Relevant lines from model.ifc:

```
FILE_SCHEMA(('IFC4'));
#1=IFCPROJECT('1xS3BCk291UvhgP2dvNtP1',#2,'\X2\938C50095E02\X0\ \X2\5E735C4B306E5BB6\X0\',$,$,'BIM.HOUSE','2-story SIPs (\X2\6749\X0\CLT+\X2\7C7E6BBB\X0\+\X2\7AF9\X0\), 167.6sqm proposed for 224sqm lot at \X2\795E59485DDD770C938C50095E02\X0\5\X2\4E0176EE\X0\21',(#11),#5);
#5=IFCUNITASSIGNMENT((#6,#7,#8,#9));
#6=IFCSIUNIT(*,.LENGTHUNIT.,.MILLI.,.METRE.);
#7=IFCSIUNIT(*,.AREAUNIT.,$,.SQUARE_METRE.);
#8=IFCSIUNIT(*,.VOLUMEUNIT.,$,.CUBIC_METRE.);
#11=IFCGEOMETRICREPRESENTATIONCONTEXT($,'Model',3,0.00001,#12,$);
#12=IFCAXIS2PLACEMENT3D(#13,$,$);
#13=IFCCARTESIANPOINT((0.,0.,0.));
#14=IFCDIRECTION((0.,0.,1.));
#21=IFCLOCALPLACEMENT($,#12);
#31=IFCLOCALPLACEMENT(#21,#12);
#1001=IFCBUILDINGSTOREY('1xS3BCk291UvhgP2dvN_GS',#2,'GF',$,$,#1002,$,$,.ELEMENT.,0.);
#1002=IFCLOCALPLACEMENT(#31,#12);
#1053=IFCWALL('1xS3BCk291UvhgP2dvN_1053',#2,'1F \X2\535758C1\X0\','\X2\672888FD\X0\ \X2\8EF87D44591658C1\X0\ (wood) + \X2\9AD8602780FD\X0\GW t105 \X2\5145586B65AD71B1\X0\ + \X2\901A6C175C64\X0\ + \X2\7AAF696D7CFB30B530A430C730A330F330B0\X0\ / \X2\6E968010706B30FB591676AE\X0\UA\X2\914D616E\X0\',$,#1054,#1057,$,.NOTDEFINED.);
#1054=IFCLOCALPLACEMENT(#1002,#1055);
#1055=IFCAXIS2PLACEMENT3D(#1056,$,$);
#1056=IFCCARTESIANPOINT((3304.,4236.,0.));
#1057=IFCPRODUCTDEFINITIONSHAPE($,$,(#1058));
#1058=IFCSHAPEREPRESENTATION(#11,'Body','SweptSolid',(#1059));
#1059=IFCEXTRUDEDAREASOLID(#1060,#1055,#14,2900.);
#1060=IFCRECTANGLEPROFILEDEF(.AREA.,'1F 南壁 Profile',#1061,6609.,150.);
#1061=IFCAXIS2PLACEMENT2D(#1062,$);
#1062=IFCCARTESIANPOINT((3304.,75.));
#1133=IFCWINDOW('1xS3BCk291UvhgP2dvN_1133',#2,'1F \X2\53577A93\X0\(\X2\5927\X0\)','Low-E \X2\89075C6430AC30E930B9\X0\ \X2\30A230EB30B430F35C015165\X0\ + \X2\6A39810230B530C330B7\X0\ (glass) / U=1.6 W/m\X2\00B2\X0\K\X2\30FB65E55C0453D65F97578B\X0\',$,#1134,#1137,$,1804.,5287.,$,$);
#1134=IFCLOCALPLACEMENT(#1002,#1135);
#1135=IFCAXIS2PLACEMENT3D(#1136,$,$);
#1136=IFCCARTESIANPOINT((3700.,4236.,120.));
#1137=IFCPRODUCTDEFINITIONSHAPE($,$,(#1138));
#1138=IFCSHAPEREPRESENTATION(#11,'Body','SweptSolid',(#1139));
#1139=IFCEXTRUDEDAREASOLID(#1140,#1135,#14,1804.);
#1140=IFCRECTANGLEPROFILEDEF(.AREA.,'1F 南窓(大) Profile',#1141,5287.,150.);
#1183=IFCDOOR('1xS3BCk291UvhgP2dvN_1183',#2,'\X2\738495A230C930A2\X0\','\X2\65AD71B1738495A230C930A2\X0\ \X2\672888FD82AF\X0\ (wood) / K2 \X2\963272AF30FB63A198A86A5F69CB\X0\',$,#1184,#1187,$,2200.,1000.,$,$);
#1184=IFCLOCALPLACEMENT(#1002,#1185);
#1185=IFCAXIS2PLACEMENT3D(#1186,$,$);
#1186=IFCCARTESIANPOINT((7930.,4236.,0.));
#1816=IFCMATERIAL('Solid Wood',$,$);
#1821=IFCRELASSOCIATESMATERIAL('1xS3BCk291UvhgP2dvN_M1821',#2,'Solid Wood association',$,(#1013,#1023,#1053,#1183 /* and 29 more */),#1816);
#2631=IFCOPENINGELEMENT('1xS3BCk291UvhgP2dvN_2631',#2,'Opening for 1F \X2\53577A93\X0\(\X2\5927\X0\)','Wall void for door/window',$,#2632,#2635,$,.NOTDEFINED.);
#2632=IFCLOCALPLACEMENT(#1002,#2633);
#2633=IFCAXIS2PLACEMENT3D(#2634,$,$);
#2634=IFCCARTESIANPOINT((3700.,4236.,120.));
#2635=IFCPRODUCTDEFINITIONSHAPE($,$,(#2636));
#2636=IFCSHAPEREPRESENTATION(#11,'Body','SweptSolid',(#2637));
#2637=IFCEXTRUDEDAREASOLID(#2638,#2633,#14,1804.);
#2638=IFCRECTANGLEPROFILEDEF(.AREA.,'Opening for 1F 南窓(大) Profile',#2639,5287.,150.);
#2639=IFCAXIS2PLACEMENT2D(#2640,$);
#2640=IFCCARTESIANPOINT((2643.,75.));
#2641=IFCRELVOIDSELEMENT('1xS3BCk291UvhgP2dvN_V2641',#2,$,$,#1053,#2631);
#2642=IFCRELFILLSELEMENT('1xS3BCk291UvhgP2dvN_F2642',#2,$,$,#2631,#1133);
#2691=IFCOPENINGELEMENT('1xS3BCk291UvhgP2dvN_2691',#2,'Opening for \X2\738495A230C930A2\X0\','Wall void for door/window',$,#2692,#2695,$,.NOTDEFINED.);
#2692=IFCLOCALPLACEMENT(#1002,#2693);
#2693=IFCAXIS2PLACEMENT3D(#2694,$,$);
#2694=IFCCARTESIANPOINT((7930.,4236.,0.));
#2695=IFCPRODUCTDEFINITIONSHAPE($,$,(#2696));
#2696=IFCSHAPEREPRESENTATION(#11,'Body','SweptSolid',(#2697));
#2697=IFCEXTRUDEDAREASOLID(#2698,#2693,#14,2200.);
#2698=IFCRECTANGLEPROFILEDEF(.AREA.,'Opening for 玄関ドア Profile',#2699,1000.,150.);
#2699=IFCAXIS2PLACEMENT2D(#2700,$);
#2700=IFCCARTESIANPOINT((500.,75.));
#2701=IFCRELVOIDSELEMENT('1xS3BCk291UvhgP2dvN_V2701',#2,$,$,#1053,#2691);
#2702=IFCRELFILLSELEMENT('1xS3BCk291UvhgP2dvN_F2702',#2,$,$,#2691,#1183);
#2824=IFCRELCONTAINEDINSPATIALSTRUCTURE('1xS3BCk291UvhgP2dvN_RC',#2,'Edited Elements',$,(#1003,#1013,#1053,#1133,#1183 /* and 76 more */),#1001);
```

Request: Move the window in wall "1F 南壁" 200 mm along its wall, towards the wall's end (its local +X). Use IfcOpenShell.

```python
import ifcopenshell
import ifcopenshell.api.geometry
import ifcopenshell.util.placement
import ifcopenshell.util.unit

model = ifcopenshell.open("model.ifc")
unit_scale = ifcopenshell.util.unit.calculate_unit_scale(model)

window = model.by_guid("1xS3BCk291UvhgP2dvN_1133")
opening = window.FillsVoids[0].RelatingOpeningElement
wall = opening.VoidsElements[0].RelatingBuildingElement

wall_matrix = ifcopenshell.util.placement.get_local_placement(wall.ObjectPlacement)
shift = wall_matrix[:3, 0] * 0.2 / unit_scale
before = ifcopenshell.util.placement.get_local_placement(window.ObjectPlacement)[:3, 3].copy()

# The window is not placed relative to its opening, so move both.
for product in (opening, window):
    matrix = ifcopenshell.util.placement.get_local_placement(product.ObjectPlacement)
    matrix[:3, 3] += shift
    ifcopenshell.api.geometry.edit_object_placement(model, product=product, matrix=matrix, is_si=False)

after = ifcopenshell.util.placement.get_local_placement(window.ObjectPlacement)[:3, 3]
print("window moved by", (after - before).round(3) + 0.0)

model.write("model-out.ifc")
```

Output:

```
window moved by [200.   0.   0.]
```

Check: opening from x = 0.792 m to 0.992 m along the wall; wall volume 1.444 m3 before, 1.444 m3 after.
